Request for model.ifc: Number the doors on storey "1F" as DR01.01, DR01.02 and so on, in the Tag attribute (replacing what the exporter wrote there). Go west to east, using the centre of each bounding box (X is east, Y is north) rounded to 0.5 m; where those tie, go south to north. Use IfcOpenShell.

First a look at what the model holds.

```python
import ifcopenshell
import ifcopenshell.util.element
import ifcopenshell.util.placement

model = ifcopenshell.open("model.ifc")
print(model.schema)
storey = next(s for s in model.by_type("IfcBuildingStorey") if s.Name == "1F")
doors = [e for e in ifcopenshell.util.element.get_decomposition(storey) if e.is_a("IfcDoor")]
for e in sorted(doors, key=lambda e: e.id()):
    origin = ifcopenshell.util.placement.get_local_placement(e.ObjectPlacement)[:3, 3]
    print(e.id(), e.Tag, e.Name, origin.round(2) + 0.0, sep=" | ")
```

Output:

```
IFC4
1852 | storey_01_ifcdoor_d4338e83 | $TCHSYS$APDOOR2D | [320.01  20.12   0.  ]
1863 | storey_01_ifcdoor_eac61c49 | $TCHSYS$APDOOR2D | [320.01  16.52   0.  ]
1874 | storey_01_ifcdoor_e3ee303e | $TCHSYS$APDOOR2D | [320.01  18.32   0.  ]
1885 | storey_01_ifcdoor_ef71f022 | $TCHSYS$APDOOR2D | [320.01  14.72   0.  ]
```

```python
import ifcopenshell
import ifcopenshell.geom
import ifcopenshell.util.element
import ifcopenshell.util.shape

model = ifcopenshell.open("model.ifc")
settings = ifcopenshell.geom.settings()
settings.set("use-world-coords", True)


def centre(element):
    shape = ifcopenshell.geom.create_shape(settings, element)
    return ifcopenshell.util.shape.get_bbox_centroid(shape.geometry)


storey = next(s for s in model.by_type("IfcBuildingStorey") if s.Name == "1F")
doors = [e for e in ifcopenshell.util.element.get_decomposition(storey) if e.is_a("IfcDoor")]

# Insertion points can sit at a corner or the storey origin, so sort by the geometry (in metres).
centres = {e: centre(e) for e in doors}
doors.sort(key=lambda e: (round(centres[e][0] / 0.5), centres[e][1]))

for i, e in enumerate(doors, start=1):
    number = f"DR01.{i:02d}"
    e.Tag = number
    print(e.id(), number)

model.write("model_v2.ifc")
```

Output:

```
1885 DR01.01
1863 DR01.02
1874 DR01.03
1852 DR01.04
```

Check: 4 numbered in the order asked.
